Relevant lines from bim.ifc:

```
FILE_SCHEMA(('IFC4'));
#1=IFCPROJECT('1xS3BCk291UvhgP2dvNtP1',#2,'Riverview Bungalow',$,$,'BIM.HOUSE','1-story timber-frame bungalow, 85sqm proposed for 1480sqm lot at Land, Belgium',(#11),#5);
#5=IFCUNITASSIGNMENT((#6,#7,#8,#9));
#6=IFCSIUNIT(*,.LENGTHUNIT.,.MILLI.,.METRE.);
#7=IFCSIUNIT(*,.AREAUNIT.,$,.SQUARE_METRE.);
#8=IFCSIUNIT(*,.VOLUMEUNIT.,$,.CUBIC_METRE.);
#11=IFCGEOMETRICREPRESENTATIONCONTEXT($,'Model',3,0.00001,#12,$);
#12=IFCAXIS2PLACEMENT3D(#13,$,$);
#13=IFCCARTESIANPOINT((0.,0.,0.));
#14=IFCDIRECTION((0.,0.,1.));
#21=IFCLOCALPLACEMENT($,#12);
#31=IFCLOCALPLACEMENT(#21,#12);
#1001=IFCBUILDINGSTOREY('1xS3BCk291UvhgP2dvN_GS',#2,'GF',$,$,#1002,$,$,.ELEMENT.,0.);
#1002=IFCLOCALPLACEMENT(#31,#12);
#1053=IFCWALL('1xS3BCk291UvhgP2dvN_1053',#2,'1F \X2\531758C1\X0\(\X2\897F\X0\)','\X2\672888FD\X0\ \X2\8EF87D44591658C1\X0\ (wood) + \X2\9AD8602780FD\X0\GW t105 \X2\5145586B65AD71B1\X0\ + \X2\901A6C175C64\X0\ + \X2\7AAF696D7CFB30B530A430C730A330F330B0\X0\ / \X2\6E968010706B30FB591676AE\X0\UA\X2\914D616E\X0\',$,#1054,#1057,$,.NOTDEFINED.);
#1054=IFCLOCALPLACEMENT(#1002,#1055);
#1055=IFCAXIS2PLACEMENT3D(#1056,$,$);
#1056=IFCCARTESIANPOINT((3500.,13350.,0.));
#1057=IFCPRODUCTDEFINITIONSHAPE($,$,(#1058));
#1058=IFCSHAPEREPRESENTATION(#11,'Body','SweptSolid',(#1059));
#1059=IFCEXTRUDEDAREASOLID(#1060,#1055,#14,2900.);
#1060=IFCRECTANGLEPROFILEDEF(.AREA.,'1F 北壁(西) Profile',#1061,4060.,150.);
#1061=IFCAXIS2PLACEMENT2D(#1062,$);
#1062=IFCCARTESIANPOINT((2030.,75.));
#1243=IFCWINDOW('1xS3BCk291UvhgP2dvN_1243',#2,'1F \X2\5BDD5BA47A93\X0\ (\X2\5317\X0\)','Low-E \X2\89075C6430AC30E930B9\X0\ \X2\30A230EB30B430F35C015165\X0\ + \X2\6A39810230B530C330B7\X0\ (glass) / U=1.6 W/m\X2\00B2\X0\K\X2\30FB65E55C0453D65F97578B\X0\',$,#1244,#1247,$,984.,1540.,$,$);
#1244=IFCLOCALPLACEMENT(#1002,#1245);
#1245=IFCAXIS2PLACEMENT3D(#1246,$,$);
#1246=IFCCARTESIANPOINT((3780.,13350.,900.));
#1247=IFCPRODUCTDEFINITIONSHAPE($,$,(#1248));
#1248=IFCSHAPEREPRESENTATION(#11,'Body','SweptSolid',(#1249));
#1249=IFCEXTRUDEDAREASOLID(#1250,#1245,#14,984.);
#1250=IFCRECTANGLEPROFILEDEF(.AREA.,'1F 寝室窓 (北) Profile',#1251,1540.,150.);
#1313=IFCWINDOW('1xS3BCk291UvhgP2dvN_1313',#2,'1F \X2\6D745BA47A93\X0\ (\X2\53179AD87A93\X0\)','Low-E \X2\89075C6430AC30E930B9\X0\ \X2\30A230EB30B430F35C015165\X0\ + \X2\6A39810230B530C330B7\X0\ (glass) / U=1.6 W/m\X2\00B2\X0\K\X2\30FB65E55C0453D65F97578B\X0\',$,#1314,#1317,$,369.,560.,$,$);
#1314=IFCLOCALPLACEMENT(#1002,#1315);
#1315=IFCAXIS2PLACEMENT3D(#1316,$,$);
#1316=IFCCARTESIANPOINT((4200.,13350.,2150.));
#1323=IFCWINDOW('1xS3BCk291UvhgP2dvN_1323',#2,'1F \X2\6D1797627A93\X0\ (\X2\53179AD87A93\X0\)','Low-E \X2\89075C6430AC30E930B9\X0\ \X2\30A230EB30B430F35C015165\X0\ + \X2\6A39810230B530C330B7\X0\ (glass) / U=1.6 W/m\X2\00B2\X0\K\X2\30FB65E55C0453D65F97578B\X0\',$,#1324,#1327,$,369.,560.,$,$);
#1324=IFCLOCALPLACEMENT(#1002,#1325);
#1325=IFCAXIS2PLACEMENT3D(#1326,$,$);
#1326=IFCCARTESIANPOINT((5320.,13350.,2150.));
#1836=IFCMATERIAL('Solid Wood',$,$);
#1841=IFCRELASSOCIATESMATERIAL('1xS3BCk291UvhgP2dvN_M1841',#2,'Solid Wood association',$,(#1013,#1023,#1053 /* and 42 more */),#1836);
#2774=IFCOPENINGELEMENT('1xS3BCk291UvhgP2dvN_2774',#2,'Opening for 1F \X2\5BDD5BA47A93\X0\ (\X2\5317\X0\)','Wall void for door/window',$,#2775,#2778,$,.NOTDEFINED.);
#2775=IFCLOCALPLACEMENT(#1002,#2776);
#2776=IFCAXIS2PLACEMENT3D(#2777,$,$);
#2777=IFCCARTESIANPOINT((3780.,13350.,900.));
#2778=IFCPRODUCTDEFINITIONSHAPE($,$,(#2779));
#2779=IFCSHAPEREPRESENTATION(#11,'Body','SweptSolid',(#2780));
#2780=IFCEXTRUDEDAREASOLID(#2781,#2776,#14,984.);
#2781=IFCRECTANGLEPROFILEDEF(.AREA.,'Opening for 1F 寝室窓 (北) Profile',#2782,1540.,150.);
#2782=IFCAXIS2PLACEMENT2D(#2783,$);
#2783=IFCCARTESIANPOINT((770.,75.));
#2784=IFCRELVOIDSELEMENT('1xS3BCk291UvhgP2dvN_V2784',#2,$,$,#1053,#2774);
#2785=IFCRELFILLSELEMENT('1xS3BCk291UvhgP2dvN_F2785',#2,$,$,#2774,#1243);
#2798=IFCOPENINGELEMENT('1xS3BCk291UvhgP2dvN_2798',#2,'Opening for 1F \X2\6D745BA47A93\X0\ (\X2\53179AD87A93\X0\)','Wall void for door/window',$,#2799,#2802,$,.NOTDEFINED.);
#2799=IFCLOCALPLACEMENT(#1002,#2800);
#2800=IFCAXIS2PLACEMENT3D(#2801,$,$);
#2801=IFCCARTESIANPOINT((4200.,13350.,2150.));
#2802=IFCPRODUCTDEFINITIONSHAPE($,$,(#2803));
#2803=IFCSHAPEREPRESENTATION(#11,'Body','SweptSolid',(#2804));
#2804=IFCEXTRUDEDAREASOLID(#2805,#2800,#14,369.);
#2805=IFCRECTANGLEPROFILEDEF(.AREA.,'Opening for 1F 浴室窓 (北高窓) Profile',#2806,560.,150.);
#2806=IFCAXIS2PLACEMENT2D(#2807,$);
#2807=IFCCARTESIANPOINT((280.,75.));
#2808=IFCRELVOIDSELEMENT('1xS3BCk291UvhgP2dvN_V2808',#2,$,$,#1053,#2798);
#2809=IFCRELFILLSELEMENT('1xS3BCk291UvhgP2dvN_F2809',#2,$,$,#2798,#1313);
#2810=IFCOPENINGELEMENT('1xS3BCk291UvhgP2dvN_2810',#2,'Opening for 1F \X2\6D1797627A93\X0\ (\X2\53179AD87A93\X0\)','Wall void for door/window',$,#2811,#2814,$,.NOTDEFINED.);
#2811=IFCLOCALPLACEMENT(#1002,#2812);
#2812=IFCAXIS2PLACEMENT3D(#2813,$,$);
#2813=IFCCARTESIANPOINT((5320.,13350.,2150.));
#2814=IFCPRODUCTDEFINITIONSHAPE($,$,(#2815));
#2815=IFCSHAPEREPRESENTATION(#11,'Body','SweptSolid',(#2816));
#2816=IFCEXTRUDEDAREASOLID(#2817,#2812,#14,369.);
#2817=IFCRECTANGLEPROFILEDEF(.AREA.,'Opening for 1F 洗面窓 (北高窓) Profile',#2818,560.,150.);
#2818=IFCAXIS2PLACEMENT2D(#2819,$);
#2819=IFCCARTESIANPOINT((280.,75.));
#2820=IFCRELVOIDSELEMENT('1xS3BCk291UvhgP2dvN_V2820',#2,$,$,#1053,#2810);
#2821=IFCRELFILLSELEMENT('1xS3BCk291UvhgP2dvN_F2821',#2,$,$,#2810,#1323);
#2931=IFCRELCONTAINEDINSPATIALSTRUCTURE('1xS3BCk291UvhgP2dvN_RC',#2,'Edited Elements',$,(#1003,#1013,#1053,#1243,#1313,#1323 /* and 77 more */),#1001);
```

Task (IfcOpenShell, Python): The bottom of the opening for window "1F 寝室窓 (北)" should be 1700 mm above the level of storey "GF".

```python
import numpy as np
import ifcopenshell
import ifcopenshell.api.geometry
import ifcopenshell.geom
import ifcopenshell.util.element
import ifcopenshell.util.placement
import ifcopenshell.util.shape
import ifcopenshell.util.unit

model = ifcopenshell.open("bim.ifc")
unit_scale = ifcopenshell.util.unit.calculate_unit_scale(model)

window = model.by_guid("1xS3BCk291UvhgP2dvN_1243")
opening = window.FillsVoids[0].RelatingOpeningElement
storey = ifcopenshell.util.element.get_container(window, ifc_class="IfcBuildingStorey")
level = ifcopenshell.util.placement.get_local_placement(storey.ObjectPlacement)[2, 3]

# The opening's origin need not be at the sill, so measure its lowest point.
shape = ifcopenshell.geom.create_shape(ifcopenshell.geom.settings(), opening)
bottom = ifcopenshell.util.shape.get_shape_bottom_elevation(shape, shape.geometry) / unit_scale
dz = level + 1700.0 - bottom

shift = np.array([0.0, 0.0, dz])
# The window is not placed relative to its opening, so move both.
for product in (opening, window):
    matrix = ifcopenshell.util.placement.get_local_placement(product.ObjectPlacement)
    matrix[:3, 3] += shift
    ifcopenshell.api.geometry.edit_object_placement(model, product=product, matrix=matrix, is_si=False)

print(f"moved by {dz * unit_scale:+.3f} m")

model.write("bim_edited.ifc")
```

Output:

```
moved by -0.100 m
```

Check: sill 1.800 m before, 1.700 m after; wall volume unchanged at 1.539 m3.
